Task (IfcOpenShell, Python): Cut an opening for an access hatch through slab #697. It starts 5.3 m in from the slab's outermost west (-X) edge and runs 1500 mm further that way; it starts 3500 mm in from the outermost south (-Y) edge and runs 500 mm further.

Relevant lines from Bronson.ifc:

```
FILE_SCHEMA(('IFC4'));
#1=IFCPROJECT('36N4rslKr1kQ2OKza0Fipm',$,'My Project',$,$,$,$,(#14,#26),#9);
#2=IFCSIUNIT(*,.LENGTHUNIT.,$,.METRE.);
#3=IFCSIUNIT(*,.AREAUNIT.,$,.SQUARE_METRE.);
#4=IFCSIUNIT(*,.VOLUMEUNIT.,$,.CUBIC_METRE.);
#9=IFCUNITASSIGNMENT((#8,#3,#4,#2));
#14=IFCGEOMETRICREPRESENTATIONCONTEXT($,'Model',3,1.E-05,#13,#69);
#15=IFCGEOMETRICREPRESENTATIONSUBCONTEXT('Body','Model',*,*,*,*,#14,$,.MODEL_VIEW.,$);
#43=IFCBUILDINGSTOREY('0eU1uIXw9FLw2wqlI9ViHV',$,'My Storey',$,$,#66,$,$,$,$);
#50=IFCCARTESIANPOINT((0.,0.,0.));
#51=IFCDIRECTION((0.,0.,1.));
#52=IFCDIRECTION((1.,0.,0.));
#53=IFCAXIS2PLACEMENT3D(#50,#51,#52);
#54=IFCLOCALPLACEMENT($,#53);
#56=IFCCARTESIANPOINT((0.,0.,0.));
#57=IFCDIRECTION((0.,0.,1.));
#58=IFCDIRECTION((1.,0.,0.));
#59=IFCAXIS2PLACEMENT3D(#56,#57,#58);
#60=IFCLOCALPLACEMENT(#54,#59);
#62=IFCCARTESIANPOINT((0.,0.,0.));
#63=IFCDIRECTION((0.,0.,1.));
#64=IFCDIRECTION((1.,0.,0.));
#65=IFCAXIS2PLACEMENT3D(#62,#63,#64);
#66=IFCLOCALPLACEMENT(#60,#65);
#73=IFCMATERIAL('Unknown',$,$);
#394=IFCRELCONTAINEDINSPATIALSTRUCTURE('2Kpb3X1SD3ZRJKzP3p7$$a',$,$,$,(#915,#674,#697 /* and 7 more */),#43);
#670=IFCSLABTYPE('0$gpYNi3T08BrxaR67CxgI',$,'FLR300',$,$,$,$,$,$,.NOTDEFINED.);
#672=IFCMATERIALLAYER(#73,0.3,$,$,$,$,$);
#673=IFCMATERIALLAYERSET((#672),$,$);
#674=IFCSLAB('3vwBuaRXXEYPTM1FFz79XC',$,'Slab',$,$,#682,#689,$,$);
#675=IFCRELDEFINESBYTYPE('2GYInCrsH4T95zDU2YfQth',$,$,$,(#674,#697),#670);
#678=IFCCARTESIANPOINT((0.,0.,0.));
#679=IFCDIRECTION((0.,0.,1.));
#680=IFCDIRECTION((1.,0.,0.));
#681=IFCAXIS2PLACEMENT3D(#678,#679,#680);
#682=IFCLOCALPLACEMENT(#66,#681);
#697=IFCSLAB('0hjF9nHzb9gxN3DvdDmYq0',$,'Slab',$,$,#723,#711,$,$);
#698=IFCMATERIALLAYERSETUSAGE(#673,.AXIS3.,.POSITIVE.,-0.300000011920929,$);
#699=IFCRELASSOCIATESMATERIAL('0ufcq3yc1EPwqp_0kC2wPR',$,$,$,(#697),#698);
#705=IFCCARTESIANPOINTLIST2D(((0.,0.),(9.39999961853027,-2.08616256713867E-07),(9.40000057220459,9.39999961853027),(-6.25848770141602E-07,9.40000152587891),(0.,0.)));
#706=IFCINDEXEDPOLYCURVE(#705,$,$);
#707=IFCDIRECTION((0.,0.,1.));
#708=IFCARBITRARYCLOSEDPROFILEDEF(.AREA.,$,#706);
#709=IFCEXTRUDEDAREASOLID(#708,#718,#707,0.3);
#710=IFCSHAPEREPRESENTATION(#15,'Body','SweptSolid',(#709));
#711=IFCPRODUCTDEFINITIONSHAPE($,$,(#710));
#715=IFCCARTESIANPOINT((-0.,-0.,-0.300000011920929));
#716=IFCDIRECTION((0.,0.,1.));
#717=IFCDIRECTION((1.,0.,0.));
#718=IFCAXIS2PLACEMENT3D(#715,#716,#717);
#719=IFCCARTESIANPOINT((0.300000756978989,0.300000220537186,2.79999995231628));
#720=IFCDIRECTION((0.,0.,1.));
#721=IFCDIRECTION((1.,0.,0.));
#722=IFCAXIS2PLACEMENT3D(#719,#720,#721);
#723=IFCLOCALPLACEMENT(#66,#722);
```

```python
import numpy as np
import ifcopenshell
import ifcopenshell.api.feature
import ifcopenshell.api.geometry
import ifcopenshell.api.root
import ifcopenshell.geom
import ifcopenshell.util.placement
import ifcopenshell.util.representation
import ifcopenshell.util.shape
import ifcopenshell.util.unit

model = ifcopenshell.open("Bronson.ifc")
unit_scale = ifcopenshell.util.unit.calculate_unit_scale(model)
settings = ifcopenshell.geom.settings()


def volume(element):
    """Net volume in cubic metres, openings subtracted."""
    shape = ifcopenshell.geom.create_shape(settings, element)
    return ifcopenshell.util.shape.get_volume(shape.geometry)


slab = model.by_guid("0hjF9nHzb9gxN3DvdDmYq0")
before = volume(slab)

# Extent in the slab's own axes, in metres. The edges named are its -X and -Y sides.
slab_shape = ifcopenshell.geom.create_shape(settings, slab)
vertices = ifcopenshell.util.shape.get_vertices(slab_shape.geometry)
x_min, y_min, bottom = vertices.min(axis=0)
top = vertices[:, 2].max()

opening = ifcopenshell.api.root.create_entity(model, ifc_class="IfcOpeningElement", name="Access hatch opening", predefined_type="OPENING")
context = ifcopenshell.util.representation.get_context(model, "Model", "Body", "MODEL_VIEW")
width, depth = 1.5, 0.5
outline = [(0.0, 0.0), (width, 0.0), (width, depth), (0.0, depth), (0.0, 0.0)]
# Overshoot both faces by 50 mm so the cut is clean.
shape = ifcopenshell.api.geometry.add_slab_representation(
    model, context=context, depth=top - bottom + 0.1, polyline=outline
)
ifcopenshell.api.geometry.assign_representation(model, product=opening, representation=shape)

matrix = ifcopenshell.util.placement.get_local_placement(slab.ObjectPlacement)
matrix[:, 3] = matrix @ np.append(np.array([x_min + 5.3, y_min + 3.5, bottom - 0.05]) / unit_scale, 1.0)
ifcopenshell.api.geometry.edit_object_placement(model, product=opening, matrix=matrix, is_si=False)
ifcopenshell.api.feature.add_feature(model, feature=opening, element=slab)

after = volume(slab)

print(f"slab volume {before:.3f} -> {after:.3f} m3")

model.write("Bronson-out.ifc")
```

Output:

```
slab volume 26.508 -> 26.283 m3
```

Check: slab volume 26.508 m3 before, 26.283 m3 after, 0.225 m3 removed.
